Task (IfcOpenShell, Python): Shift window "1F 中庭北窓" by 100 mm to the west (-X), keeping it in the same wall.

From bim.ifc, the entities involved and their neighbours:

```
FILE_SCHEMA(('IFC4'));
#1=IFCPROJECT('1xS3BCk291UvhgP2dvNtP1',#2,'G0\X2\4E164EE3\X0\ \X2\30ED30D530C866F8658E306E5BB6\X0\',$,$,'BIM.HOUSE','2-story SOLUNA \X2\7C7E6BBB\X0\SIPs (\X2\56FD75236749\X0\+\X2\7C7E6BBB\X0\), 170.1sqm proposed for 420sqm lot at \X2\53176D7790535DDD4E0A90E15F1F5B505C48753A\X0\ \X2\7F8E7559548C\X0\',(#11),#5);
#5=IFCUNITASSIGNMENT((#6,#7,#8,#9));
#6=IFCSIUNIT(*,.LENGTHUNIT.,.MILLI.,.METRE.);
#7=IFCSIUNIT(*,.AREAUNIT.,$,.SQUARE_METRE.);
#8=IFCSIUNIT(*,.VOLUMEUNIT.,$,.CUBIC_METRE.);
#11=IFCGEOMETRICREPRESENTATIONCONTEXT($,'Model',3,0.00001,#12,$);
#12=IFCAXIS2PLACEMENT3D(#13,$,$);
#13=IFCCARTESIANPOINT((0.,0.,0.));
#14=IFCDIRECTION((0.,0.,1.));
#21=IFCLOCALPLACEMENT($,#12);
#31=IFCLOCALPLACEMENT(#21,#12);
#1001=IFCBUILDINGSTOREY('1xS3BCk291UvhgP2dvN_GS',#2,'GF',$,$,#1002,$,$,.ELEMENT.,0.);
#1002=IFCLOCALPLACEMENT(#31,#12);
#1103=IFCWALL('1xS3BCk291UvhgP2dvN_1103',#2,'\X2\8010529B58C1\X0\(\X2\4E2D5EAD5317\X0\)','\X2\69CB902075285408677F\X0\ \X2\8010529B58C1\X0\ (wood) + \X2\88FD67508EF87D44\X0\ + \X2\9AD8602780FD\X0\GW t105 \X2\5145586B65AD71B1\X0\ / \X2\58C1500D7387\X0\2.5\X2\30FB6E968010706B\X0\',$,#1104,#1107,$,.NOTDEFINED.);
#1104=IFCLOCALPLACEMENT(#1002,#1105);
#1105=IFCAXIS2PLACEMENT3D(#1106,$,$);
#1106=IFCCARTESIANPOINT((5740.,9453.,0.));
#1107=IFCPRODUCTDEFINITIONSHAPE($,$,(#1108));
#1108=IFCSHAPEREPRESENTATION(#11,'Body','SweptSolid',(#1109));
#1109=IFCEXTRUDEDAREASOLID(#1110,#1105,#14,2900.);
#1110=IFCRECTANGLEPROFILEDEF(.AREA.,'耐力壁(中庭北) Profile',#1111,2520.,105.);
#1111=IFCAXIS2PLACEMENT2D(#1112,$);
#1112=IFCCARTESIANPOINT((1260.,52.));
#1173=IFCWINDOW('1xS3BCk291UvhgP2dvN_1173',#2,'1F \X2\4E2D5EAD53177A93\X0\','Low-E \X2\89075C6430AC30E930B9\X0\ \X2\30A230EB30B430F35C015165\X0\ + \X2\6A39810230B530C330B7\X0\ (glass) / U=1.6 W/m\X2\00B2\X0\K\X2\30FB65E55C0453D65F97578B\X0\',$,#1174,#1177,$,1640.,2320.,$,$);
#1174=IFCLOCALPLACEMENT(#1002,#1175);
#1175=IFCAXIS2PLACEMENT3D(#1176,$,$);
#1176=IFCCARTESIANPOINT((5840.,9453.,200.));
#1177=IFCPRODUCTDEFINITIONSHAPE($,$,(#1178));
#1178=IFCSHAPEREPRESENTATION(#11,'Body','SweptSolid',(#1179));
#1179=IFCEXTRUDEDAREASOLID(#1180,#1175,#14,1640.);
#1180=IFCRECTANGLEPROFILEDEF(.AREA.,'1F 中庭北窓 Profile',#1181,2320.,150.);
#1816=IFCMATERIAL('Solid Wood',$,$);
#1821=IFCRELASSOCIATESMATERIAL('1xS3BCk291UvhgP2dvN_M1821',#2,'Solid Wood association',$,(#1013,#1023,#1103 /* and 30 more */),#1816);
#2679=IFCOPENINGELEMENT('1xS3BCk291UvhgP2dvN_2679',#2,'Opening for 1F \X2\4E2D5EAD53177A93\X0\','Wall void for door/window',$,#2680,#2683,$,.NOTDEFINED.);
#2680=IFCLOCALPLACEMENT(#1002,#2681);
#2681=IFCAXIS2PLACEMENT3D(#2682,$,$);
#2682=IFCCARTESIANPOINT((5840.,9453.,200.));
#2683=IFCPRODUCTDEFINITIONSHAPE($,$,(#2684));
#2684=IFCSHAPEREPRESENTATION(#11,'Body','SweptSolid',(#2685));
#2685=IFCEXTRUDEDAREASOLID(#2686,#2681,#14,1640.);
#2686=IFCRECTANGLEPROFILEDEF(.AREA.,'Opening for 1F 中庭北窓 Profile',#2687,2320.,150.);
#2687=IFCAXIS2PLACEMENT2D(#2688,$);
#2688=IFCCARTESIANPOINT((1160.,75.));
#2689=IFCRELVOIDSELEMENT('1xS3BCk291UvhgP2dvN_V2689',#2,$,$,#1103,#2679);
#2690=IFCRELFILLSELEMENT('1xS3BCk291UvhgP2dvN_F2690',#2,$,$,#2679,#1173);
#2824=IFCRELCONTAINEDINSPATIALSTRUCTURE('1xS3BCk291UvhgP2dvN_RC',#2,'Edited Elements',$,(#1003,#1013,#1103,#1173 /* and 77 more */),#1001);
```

```python
import ifcopenshell
import ifcopenshell.api.geometry
import ifcopenshell.util.placement
import ifcopenshell.util.unit

model = ifcopenshell.open("bim.ifc")
unit_scale = ifcopenshell.util.unit.calculate_unit_scale(model)

window = model.by_guid("1xS3BCk291UvhgP2dvN_1173")
opening = window.FillsVoids[0].RelatingOpeningElement
wall = opening.VoidsElements[0].RelatingBuildingElement

wall_matrix = ifcopenshell.util.placement.get_local_placement(wall.ObjectPlacement)
shift = wall_matrix[:3, 0] * -0.1 / unit_scale
before = ifcopenshell.util.placement.get_local_placement(window.ObjectPlacement)[:3, 3].copy()

# The window is not placed relative to its opening, so move both.
for product in (opening, window):
    matrix = ifcopenshell.util.placement.get_local_placement(product.ObjectPlacement)
    matrix[:3, 3] += shift
    ifcopenshell.api.geometry.edit_object_placement(model, product=product, matrix=matrix, is_si=False)

after = ifcopenshell.util.placement.get_local_placement(window.ObjectPlacement)[:3, 3]
print("window moved by", (after - before).round(3) + 0.0)

model.write("bim-out.ifc")
```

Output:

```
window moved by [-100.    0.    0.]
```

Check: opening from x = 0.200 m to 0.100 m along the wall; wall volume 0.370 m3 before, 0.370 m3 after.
